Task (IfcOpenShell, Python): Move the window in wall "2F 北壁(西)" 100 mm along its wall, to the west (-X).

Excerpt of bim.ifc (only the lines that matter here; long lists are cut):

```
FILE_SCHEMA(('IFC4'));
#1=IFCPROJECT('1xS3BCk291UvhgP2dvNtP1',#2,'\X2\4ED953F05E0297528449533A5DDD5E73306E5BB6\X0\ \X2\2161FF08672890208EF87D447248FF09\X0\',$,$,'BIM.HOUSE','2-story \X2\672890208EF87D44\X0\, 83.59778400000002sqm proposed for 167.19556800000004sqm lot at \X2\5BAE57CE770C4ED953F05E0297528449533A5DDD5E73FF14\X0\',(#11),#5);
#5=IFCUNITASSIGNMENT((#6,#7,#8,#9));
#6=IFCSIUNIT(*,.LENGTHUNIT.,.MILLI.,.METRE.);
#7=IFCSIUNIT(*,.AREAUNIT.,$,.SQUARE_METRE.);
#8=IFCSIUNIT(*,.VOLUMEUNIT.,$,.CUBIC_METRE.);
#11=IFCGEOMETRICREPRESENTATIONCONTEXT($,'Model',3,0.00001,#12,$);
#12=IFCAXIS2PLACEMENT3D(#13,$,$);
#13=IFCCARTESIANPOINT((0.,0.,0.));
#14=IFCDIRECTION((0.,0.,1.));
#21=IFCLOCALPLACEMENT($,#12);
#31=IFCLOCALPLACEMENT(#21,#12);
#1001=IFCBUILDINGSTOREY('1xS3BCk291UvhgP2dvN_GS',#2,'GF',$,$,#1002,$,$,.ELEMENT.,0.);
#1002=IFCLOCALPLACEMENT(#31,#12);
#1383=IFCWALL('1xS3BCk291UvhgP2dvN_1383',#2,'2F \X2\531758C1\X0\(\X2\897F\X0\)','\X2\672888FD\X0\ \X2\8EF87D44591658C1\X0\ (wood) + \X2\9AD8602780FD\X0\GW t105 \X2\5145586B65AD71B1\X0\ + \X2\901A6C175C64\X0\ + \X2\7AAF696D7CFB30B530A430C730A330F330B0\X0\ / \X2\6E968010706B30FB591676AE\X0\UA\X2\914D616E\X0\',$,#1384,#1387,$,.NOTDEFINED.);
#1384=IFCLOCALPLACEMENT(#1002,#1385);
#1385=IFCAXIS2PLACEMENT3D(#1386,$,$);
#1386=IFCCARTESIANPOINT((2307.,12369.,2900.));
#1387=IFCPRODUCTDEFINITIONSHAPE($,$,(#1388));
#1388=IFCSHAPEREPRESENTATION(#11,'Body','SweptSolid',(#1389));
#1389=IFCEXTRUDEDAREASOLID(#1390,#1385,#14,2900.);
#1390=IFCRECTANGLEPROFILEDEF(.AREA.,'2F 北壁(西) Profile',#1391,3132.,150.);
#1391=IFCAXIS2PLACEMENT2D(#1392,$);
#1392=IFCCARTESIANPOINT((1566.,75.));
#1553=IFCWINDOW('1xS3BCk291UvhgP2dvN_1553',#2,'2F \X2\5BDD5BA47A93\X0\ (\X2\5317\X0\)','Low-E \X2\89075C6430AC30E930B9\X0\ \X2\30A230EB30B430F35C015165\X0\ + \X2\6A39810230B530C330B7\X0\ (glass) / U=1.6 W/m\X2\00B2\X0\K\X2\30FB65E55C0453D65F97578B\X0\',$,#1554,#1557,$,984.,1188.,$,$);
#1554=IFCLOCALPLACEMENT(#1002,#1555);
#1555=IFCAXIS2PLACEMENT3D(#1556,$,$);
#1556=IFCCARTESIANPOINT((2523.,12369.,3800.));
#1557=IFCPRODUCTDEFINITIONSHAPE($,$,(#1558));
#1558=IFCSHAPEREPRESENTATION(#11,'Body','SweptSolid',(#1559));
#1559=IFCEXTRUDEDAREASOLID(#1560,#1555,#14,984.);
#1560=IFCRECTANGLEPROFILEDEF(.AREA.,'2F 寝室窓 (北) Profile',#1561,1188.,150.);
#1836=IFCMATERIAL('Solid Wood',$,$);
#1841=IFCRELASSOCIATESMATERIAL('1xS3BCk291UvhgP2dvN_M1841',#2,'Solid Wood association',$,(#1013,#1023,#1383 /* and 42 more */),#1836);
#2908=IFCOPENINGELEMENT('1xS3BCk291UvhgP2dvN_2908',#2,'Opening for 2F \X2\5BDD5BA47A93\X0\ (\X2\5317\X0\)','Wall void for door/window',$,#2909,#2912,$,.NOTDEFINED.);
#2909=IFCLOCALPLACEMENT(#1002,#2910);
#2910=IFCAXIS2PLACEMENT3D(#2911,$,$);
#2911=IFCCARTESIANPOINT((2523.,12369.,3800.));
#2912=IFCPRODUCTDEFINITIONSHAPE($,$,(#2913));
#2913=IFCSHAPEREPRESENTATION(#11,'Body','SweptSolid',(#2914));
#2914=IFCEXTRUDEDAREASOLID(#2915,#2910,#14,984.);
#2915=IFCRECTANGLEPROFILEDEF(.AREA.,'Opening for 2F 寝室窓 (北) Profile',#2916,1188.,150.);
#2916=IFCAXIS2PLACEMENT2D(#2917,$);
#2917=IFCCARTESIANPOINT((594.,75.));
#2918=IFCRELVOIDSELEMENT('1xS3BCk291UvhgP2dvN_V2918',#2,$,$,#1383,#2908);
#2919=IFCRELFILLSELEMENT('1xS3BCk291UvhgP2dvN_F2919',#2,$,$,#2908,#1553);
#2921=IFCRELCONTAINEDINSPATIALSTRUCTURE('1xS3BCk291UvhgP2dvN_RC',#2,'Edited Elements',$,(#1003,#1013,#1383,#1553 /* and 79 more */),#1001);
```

```python
import ifcopenshell
import ifcopenshell.api.geometry
import ifcopenshell.util.placement

model = ifcopenshell.open("bim.ifc")

window = model.by_guid("1xS3BCk291UvhgP2dvN_1553")
opening = window.FillsVoids[0].RelatingOpeningElement
wall = opening.VoidsElements[0].RelatingBuildingElement

wall_matrix = ifcopenshell.util.placement.get_local_placement(wall.ObjectPlacement)
shift = wall_matrix[:3, 0] * -100.0
before = ifcopenshell.util.placement.get_local_placement(window.ObjectPlacement)[:3, 3].copy()

# The window is not placed relative to its opening, so move both.
for product in (opening, window):
    matrix = ifcopenshell.util.placement.get_local_placement(product.ObjectPlacement)
    matrix[:3, 3] += shift
    ifcopenshell.api.geometry.edit_object_placement(model, product=product, matrix=matrix, is_si=False)

after = ifcopenshell.util.placement.get_local_placement(window.ObjectPlacement)[:3, 3]
print("window moved by", (after - before).round(3) + 0.0)

model.write("bim_rev.ifc")
```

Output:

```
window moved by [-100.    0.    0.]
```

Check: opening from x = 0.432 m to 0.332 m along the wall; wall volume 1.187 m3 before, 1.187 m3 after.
